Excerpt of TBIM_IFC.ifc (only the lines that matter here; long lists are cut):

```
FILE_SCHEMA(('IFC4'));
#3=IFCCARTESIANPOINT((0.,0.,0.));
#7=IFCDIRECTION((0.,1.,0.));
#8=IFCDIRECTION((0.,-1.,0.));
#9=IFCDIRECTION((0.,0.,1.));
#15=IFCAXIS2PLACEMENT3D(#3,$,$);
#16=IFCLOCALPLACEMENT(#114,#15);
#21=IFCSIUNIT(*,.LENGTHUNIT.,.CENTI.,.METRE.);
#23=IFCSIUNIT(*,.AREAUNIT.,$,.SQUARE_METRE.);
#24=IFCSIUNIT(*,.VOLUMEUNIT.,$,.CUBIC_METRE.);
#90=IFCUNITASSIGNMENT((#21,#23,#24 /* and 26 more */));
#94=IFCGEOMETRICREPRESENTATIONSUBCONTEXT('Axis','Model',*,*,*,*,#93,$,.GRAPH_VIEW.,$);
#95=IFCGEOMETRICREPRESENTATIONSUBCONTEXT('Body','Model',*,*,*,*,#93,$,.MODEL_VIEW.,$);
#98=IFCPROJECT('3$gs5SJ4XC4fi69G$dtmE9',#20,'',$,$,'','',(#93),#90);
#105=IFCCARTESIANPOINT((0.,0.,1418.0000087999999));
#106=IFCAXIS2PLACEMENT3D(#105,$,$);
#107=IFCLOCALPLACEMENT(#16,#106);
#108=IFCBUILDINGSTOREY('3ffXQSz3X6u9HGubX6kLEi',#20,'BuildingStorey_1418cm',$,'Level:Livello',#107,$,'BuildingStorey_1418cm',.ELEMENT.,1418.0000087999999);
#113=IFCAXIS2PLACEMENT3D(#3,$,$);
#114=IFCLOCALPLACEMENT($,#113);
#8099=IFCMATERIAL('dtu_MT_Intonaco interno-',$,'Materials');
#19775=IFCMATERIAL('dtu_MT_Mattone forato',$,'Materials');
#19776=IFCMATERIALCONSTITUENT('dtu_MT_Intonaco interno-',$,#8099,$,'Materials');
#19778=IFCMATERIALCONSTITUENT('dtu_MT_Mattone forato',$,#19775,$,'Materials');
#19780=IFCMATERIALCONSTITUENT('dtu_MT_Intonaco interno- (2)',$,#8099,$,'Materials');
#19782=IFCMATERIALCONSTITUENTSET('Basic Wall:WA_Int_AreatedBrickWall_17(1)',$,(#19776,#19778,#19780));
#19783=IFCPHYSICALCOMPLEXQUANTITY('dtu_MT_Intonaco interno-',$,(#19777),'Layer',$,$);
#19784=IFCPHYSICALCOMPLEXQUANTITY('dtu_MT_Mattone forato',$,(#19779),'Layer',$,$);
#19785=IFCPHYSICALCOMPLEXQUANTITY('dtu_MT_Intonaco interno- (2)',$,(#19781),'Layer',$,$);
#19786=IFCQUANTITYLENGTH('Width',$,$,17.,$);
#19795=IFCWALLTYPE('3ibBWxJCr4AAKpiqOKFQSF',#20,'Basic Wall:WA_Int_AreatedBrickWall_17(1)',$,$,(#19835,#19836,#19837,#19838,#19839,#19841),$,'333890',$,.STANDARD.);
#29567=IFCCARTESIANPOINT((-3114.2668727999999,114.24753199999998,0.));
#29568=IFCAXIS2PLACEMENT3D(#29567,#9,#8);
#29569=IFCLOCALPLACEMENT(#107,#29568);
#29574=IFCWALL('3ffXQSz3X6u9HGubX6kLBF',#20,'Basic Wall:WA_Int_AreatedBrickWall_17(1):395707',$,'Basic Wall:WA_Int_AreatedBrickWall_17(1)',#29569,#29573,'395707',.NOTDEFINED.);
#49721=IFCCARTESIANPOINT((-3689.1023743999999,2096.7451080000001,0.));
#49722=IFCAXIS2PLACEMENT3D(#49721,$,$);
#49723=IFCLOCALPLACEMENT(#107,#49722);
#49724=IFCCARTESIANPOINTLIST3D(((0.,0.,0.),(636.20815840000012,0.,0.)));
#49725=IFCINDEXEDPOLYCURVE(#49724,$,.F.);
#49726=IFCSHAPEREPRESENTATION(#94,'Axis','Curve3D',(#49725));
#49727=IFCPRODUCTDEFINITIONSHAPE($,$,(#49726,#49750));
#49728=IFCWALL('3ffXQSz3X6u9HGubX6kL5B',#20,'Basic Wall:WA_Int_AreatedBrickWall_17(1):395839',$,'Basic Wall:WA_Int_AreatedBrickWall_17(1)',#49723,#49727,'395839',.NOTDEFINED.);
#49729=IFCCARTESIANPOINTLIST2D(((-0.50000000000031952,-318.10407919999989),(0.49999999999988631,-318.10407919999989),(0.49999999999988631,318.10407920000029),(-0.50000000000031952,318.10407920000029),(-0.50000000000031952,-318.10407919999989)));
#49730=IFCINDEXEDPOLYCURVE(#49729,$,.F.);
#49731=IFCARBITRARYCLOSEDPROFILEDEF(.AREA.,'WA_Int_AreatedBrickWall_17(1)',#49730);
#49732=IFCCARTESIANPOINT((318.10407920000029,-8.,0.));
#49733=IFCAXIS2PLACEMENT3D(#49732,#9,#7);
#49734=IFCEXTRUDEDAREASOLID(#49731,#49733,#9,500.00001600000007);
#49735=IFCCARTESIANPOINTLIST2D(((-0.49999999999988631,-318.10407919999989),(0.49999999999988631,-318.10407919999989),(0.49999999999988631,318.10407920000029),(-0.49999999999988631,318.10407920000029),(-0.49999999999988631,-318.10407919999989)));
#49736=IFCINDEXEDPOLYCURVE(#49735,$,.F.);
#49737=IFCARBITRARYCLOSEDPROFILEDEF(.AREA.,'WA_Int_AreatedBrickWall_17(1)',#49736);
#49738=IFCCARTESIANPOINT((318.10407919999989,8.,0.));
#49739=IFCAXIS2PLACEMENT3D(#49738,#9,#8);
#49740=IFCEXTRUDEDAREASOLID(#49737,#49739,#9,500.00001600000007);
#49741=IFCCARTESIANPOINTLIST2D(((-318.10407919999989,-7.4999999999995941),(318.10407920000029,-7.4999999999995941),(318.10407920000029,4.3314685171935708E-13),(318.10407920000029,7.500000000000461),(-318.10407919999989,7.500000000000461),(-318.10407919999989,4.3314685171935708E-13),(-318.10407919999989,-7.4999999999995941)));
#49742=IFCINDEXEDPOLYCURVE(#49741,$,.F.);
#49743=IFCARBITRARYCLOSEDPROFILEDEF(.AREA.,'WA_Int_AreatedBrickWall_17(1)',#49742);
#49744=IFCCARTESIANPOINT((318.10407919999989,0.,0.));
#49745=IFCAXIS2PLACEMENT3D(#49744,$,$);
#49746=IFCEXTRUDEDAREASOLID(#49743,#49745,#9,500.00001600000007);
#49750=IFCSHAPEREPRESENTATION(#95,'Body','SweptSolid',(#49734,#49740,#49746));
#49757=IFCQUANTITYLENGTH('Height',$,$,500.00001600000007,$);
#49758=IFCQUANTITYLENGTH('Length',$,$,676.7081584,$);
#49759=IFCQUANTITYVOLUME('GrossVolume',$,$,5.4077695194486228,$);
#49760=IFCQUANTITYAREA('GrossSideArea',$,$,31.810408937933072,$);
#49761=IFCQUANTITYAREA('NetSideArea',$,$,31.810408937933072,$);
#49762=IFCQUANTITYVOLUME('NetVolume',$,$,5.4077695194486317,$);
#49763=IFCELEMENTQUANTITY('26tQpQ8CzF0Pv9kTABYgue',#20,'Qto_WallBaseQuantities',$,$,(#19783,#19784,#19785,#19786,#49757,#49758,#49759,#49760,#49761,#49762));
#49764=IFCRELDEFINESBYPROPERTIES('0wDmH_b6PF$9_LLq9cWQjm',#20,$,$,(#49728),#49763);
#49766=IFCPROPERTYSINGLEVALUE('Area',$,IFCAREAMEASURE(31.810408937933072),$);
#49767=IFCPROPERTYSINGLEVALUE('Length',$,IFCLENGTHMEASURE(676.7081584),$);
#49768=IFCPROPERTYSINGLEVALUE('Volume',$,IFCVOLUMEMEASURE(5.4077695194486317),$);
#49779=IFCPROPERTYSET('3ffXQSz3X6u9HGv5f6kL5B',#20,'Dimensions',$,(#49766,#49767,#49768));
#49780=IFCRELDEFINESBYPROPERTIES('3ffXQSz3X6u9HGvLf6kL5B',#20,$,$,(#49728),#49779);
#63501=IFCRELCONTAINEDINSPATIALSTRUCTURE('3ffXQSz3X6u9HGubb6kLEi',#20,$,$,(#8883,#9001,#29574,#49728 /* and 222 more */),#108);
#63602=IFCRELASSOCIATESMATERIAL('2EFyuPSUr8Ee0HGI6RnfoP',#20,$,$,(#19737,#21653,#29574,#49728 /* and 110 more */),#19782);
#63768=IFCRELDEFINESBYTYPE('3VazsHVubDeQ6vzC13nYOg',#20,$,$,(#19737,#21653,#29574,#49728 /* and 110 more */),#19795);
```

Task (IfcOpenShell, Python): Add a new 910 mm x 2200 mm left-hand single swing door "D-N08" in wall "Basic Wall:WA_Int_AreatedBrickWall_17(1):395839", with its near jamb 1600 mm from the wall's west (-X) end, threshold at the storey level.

```python
import numpy as np
import ifcopenshell
import ifcopenshell.api.feature
import ifcopenshell.api.geometry
import ifcopenshell.api.pset
import ifcopenshell.api.root
import ifcopenshell.api.spatial
import ifcopenshell.geom
import ifcopenshell.util.element
import ifcopenshell.util.placement
import ifcopenshell.util.representation
import ifcopenshell.util.shape
import ifcopenshell.util.unit

model = ifcopenshell.open("TBIM_IFC.ifc")
unit_scale = ifcopenshell.util.unit.calculate_unit_scale(model)
area_scale = ifcopenshell.util.unit.calculate_unit_scale(model, "AREAUNIT")
volume_scale = ifcopenshell.util.unit.calculate_unit_scale(model, "VOLUMEUNIT")
settings = ifcopenshell.geom.settings()


def volume(element):
    """Net volume in cubic metres, openings subtracted."""
    shape = ifcopenshell.geom.create_shape(settings, element)
    return ifcopenshell.util.shape.get_volume(shape.geometry)


wall = model.by_id(49728)
storey = ifcopenshell.util.element.get_container(wall, ifc_class="IfcBuildingStorey")
context = ifcopenshell.util.representation.get_context(model, "Model", "Body", "MODEL_VIEW")
before = volume(wall)

width, height, from_end, sill = 0.91, 2.2, 1.6, 0.0  # metres

# The wall runs along its own X axis, and the end named is its -X end.
wall_shape = ifcopenshell.geom.create_shape(settings, wall)
x, y, z = ifcopenshell.util.shape.get_vertices(wall_shape.geometry).T
start = x.min() + from_end
face, thickness = float(y.min()), float(y.max() - y.min())
wall_matrix = ifcopenshell.util.placement.get_local_placement(wall.ObjectPlacement)
level = ifcopenshell.util.placement.get_local_placement(storey.ObjectPlacement)[2, 3]


def in_wall(x, y):
    """Placement at x, y metres in the wall's axes, at sill height."""
    matrix = wall_matrix.copy()
    matrix[:, 3] = wall_matrix @ np.array([x / unit_scale, y / unit_scale, 0.0, 1.0])
    matrix[2, 3] = level + sill / unit_scale
    return matrix


# Opening: a box that overshoots both wall faces by 50 mm.
opening = ifcopenshell.api.root.create_entity(model, ifc_class="IfcOpeningElement", predefined_type="OPENING")
box = ifcopenshell.api.geometry.add_wall_representation(
    model, context=context, length=width, height=height, thickness=thickness + 0.1
)
ifcopenshell.api.geometry.assign_representation(model, product=opening, representation=box)
ifcopenshell.api.geometry.edit_object_placement(model, product=opening, matrix=in_wall(start, face - 0.05), is_si=False)
ifcopenshell.api.feature.add_feature(model, feature=opening, element=wall)

door = ifcopenshell.api.root.create_entity(model, ifc_class="IfcDoor", name="D-N08", predefined_type="DOOR")
door.OverallWidth, door.OverallHeight = width / unit_scale, height / unit_scale
door.OperationType = "SINGLE_SWING_LEFT"
body = ifcopenshell.api.geometry.add_door_representation(
    model,
    context=context,
    overall_width=door.OverallWidth,
    overall_height=door.OverallHeight,
    operation_type="SINGLE_SWING_LEFT",
    lining_properties={"LiningDepth": thickness / unit_scale, "ThresholdDepth": thickness / unit_scale},
)
ifcopenshell.api.geometry.assign_representation(model, product=door, representation=body)
ifcopenshell.api.spatial.assign_container(model, products=[door], relating_structure=storey)
ifcopenshell.api.feature.add_filling(model, opening=opening, element=door)

# The lining spans the wall, so the door starts at the wall face.
ifcopenshell.api.geometry.edit_object_placement(model, product=door, matrix=in_wall(start, face), is_si=False)

after = volume(wall)

# Update the wall's stored quantities.
qto = model.by_id(ifcopenshell.util.element.get_pset(wall, "Qto_WallBaseQuantities", should_inherit=False)["id"])
ifcopenshell.api.pset.edit_qto(model, qto=qto, properties={
    "NetSideArea": after / thickness / area_scale,
    "NetVolume": after / volume_scale,
})
pset = model.by_id(ifcopenshell.util.element.get_pset(wall, "Dimensions", should_inherit=False)["id"])
ifcopenshell.api.pset.edit_pset(model, pset=pset, properties={
    "Area": model.create_entity("IfcAreaMeasure", after / thickness / area_scale),
    "Volume": model.create_entity("IfcVolumeMeasure", after / volume_scale),
})

print(f"wall volume {before:.3f} -> {after:.3f} m3")

model.write("TBIM_IFC_rev.ifc")
```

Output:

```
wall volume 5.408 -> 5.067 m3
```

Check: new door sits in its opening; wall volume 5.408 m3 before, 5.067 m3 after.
